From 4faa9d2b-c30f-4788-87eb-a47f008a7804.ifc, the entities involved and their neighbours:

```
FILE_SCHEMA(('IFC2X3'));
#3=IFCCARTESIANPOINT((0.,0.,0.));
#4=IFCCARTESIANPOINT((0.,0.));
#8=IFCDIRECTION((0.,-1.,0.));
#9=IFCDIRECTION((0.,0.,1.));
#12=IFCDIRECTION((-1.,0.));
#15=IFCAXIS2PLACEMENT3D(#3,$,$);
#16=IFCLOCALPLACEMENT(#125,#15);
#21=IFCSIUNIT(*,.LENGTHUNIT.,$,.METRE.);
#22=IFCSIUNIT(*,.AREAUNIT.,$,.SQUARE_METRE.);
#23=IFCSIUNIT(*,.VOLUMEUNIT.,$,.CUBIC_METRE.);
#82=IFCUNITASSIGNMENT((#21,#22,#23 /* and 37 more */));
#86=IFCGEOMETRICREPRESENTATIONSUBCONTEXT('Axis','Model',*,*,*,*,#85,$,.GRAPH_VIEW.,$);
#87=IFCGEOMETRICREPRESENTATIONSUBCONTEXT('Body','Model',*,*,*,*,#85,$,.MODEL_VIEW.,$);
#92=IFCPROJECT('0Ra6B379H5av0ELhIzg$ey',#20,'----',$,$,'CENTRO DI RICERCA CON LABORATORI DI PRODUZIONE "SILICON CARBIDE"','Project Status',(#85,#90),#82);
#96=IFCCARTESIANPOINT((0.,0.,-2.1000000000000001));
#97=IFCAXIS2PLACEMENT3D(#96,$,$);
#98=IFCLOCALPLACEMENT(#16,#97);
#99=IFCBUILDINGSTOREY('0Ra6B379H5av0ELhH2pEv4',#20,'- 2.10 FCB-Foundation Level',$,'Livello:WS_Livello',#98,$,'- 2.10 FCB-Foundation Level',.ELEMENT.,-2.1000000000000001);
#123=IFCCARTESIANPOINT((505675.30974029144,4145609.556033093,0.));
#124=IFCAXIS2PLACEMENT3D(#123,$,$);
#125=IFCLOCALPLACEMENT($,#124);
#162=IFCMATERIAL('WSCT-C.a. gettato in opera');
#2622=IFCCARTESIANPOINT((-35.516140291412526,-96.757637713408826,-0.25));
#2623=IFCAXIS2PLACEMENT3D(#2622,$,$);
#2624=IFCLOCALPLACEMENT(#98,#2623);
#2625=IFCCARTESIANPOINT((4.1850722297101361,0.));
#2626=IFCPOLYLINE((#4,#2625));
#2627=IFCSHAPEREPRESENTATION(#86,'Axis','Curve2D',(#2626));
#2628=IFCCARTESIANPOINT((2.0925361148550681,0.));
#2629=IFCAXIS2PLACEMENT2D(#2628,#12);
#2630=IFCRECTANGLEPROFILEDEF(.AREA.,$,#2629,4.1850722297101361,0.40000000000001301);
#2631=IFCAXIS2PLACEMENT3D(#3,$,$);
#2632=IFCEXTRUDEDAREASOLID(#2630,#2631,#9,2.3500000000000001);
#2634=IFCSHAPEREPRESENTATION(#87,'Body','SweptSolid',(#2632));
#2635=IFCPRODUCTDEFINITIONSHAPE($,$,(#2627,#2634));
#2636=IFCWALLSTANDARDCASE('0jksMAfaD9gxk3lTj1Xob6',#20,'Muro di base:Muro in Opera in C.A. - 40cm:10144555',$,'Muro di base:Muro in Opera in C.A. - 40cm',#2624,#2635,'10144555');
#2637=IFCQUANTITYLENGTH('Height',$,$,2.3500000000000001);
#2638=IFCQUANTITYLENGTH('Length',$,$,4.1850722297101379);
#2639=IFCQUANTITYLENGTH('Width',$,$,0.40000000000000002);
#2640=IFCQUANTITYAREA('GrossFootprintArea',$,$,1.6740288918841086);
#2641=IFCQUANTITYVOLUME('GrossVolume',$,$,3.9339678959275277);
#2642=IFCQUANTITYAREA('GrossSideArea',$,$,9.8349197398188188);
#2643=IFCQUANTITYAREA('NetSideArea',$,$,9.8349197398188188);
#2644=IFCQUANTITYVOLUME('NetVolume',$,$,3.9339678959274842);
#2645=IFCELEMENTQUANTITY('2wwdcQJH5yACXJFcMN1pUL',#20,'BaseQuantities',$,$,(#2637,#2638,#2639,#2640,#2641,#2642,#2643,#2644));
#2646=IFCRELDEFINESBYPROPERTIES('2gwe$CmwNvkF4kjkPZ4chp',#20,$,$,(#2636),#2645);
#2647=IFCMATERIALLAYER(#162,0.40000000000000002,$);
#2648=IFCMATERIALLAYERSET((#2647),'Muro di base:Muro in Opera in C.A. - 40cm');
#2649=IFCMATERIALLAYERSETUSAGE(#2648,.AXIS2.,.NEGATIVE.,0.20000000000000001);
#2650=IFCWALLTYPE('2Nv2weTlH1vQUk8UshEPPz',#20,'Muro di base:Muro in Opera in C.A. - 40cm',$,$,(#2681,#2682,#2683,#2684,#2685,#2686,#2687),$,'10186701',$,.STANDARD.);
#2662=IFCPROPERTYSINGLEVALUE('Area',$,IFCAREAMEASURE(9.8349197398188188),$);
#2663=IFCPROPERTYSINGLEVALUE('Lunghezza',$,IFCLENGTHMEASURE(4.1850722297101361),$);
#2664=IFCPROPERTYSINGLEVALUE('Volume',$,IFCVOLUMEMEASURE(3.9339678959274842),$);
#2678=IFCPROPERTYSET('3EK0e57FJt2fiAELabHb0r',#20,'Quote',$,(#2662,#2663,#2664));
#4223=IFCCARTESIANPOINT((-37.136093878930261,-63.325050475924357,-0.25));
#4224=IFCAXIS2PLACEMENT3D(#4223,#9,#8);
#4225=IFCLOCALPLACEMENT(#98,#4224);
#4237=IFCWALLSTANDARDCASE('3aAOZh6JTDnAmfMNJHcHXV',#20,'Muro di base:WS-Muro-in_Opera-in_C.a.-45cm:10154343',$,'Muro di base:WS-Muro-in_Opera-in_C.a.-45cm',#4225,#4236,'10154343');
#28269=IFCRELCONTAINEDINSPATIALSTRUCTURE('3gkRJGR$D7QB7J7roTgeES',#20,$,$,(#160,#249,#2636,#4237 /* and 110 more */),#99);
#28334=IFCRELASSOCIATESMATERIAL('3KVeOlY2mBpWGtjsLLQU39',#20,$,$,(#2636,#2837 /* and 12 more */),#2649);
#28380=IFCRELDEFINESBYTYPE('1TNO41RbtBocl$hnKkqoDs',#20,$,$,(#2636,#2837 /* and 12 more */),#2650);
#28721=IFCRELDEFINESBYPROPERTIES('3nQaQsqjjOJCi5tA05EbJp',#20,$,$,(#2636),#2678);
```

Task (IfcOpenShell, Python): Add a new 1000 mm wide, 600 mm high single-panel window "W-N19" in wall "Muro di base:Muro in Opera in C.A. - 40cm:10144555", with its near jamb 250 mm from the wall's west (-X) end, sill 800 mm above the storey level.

```python
import numpy as np
import ifcopenshell
import ifcopenshell.api.feature
import ifcopenshell.api.geometry
import ifcopenshell.api.pset
import ifcopenshell.api.root
import ifcopenshell.api.spatial
import ifcopenshell.api.type
import ifcopenshell.geom
import ifcopenshell.util.element
import ifcopenshell.util.placement
import ifcopenshell.util.representation
import ifcopenshell.util.shape
import ifcopenshell.util.unit

model = ifcopenshell.open("4faa9d2b-c30f-4788-87eb-a47f008a7804.ifc")
unit_scale = ifcopenshell.util.unit.calculate_unit_scale(model)
area_scale = ifcopenshell.util.unit.calculate_unit_scale(model, "AREAUNIT")
volume_scale = ifcopenshell.util.unit.calculate_unit_scale(model, "VOLUMEUNIT")
settings = ifcopenshell.geom.settings()


def volume(element):
    """Net volume in cubic metres, openings subtracted."""
    shape = ifcopenshell.geom.create_shape(settings, element)
    return ifcopenshell.util.shape.get_volume(shape.geometry)


wall = model.by_id(2636)
storey = ifcopenshell.util.element.get_container(wall, ifc_class="IfcBuildingStorey")
context = ifcopenshell.util.representation.get_context(model, "Model", "Body", "MODEL_VIEW")
before = volume(wall)

width, height, from_end, sill = 1, 0.6, 0.25, 0.8  # metres

# The wall runs along its own X axis, and the end named is its -X end.
wall_shape = ifcopenshell.geom.create_shape(settings, wall)
x, y, z = ifcopenshell.util.shape.get_vertices(wall_shape.geometry).T
start = x.min() + from_end
face, thickness = float(y.min()), float(y.max() - y.min())
wall_matrix = ifcopenshell.util.placement.get_local_placement(wall.ObjectPlacement)
level = ifcopenshell.util.placement.get_local_placement(storey.ObjectPlacement)[2, 3]


def in_wall(x, y):
    """Placement at x, y metres in the wall's axes, at sill height."""
    matrix = wall_matrix.copy()
    matrix[:, 3] = wall_matrix @ np.array([x / unit_scale, y / unit_scale, 0.0, 1.0])
    matrix[2, 3] = level + sill / unit_scale
    return matrix


# Opening: a box that overshoots both wall faces by 50 mm.
opening = ifcopenshell.api.root.create_entity(model, ifc_class="IfcOpeningElement")
box = ifcopenshell.api.geometry.add_wall_representation(
    model, context=context, length=width, height=height, thickness=thickness + 0.1
)
ifcopenshell.api.geometry.assign_representation(model, product=opening, representation=box)
ifcopenshell.api.geometry.edit_object_placement(model, product=opening, matrix=in_wall(start, face - 0.05), is_si=False)
ifcopenshell.api.feature.add_feature(model, feature=opening, element=wall)

window = ifcopenshell.api.root.create_entity(model, ifc_class="IfcWindow", name="W-N19")
window.OverallWidth, window.OverallHeight = width / unit_scale, height / unit_scale
body = ifcopenshell.api.geometry.add_window_representation(
    model,
    context=context,
    overall_width=window.OverallWidth,
    overall_height=window.OverallHeight,
    partition_type="SINGLE_PANEL",
)
ifcopenshell.api.geometry.assign_representation(model, product=window, representation=body)
ifcopenshell.api.spatial.assign_container(model, products=[window], relating_structure=storey)
fills = ifcopenshell.api.feature.add_filling(model, opening=opening, element=window)
fills.OwnerHistory = window.OwnerHistory  # required in IFC2X3

# IFC2X3 keeps the operation on the window style.
style = ifcopenshell.api.root.create_entity(model, ifc_class="IfcWindowStyle", name="W-N19")
style.OperationType, style.ConstructionType = "SINGLE_PANEL", "NOTDEFINED"
style.ParameterTakesPrecedence = style.Sizeable = False
ifcopenshell.api.type.assign_type(model, related_objects=[window], relating_type=style)

# Centre the window in the wall's thickness.
ifcopenshell.api.geometry.edit_object_placement(model, product=window, matrix=in_wall(start, face), is_si=False)
window_shape = ifcopenshell.geom.create_shape(settings, window)
depth = ifcopenshell.util.shape.get_vertices(window_shape.geometry)[:, 1]
offset = face + thickness / 2 - (depth.min() + depth.max()) / 2
ifcopenshell.api.geometry.edit_object_placement(model, product=window, matrix=in_wall(start, offset), is_si=False)

after = volume(wall)

# Update the wall's stored quantities.
qto = model.by_id(ifcopenshell.util.element.get_pset(wall, "BaseQuantities", should_inherit=False)["id"])
ifcopenshell.api.pset.edit_qto(model, qto=qto, properties={
    "NetSideArea": after / thickness / area_scale,
    "NetVolume": after / volume_scale,
})
pset = model.by_id(ifcopenshell.util.element.get_pset(wall, "Quote", should_inherit=False)["id"])
ifcopenshell.api.pset.edit_pset(model, pset=pset, properties={
    "Area": model.create_entity("IfcAreaMeasure", after / thickness / area_scale),
    "Volume": model.create_entity("IfcVolumeMeasure", after / volume_scale),
})

print(f"wall volume {before:.3f} -> {after:.3f} m3")

model.write("4faa9d2b-c30f-4788-87eb-a47f008a7804_updated.ifc")
```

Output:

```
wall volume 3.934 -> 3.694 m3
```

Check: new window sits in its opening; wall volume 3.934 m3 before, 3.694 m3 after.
